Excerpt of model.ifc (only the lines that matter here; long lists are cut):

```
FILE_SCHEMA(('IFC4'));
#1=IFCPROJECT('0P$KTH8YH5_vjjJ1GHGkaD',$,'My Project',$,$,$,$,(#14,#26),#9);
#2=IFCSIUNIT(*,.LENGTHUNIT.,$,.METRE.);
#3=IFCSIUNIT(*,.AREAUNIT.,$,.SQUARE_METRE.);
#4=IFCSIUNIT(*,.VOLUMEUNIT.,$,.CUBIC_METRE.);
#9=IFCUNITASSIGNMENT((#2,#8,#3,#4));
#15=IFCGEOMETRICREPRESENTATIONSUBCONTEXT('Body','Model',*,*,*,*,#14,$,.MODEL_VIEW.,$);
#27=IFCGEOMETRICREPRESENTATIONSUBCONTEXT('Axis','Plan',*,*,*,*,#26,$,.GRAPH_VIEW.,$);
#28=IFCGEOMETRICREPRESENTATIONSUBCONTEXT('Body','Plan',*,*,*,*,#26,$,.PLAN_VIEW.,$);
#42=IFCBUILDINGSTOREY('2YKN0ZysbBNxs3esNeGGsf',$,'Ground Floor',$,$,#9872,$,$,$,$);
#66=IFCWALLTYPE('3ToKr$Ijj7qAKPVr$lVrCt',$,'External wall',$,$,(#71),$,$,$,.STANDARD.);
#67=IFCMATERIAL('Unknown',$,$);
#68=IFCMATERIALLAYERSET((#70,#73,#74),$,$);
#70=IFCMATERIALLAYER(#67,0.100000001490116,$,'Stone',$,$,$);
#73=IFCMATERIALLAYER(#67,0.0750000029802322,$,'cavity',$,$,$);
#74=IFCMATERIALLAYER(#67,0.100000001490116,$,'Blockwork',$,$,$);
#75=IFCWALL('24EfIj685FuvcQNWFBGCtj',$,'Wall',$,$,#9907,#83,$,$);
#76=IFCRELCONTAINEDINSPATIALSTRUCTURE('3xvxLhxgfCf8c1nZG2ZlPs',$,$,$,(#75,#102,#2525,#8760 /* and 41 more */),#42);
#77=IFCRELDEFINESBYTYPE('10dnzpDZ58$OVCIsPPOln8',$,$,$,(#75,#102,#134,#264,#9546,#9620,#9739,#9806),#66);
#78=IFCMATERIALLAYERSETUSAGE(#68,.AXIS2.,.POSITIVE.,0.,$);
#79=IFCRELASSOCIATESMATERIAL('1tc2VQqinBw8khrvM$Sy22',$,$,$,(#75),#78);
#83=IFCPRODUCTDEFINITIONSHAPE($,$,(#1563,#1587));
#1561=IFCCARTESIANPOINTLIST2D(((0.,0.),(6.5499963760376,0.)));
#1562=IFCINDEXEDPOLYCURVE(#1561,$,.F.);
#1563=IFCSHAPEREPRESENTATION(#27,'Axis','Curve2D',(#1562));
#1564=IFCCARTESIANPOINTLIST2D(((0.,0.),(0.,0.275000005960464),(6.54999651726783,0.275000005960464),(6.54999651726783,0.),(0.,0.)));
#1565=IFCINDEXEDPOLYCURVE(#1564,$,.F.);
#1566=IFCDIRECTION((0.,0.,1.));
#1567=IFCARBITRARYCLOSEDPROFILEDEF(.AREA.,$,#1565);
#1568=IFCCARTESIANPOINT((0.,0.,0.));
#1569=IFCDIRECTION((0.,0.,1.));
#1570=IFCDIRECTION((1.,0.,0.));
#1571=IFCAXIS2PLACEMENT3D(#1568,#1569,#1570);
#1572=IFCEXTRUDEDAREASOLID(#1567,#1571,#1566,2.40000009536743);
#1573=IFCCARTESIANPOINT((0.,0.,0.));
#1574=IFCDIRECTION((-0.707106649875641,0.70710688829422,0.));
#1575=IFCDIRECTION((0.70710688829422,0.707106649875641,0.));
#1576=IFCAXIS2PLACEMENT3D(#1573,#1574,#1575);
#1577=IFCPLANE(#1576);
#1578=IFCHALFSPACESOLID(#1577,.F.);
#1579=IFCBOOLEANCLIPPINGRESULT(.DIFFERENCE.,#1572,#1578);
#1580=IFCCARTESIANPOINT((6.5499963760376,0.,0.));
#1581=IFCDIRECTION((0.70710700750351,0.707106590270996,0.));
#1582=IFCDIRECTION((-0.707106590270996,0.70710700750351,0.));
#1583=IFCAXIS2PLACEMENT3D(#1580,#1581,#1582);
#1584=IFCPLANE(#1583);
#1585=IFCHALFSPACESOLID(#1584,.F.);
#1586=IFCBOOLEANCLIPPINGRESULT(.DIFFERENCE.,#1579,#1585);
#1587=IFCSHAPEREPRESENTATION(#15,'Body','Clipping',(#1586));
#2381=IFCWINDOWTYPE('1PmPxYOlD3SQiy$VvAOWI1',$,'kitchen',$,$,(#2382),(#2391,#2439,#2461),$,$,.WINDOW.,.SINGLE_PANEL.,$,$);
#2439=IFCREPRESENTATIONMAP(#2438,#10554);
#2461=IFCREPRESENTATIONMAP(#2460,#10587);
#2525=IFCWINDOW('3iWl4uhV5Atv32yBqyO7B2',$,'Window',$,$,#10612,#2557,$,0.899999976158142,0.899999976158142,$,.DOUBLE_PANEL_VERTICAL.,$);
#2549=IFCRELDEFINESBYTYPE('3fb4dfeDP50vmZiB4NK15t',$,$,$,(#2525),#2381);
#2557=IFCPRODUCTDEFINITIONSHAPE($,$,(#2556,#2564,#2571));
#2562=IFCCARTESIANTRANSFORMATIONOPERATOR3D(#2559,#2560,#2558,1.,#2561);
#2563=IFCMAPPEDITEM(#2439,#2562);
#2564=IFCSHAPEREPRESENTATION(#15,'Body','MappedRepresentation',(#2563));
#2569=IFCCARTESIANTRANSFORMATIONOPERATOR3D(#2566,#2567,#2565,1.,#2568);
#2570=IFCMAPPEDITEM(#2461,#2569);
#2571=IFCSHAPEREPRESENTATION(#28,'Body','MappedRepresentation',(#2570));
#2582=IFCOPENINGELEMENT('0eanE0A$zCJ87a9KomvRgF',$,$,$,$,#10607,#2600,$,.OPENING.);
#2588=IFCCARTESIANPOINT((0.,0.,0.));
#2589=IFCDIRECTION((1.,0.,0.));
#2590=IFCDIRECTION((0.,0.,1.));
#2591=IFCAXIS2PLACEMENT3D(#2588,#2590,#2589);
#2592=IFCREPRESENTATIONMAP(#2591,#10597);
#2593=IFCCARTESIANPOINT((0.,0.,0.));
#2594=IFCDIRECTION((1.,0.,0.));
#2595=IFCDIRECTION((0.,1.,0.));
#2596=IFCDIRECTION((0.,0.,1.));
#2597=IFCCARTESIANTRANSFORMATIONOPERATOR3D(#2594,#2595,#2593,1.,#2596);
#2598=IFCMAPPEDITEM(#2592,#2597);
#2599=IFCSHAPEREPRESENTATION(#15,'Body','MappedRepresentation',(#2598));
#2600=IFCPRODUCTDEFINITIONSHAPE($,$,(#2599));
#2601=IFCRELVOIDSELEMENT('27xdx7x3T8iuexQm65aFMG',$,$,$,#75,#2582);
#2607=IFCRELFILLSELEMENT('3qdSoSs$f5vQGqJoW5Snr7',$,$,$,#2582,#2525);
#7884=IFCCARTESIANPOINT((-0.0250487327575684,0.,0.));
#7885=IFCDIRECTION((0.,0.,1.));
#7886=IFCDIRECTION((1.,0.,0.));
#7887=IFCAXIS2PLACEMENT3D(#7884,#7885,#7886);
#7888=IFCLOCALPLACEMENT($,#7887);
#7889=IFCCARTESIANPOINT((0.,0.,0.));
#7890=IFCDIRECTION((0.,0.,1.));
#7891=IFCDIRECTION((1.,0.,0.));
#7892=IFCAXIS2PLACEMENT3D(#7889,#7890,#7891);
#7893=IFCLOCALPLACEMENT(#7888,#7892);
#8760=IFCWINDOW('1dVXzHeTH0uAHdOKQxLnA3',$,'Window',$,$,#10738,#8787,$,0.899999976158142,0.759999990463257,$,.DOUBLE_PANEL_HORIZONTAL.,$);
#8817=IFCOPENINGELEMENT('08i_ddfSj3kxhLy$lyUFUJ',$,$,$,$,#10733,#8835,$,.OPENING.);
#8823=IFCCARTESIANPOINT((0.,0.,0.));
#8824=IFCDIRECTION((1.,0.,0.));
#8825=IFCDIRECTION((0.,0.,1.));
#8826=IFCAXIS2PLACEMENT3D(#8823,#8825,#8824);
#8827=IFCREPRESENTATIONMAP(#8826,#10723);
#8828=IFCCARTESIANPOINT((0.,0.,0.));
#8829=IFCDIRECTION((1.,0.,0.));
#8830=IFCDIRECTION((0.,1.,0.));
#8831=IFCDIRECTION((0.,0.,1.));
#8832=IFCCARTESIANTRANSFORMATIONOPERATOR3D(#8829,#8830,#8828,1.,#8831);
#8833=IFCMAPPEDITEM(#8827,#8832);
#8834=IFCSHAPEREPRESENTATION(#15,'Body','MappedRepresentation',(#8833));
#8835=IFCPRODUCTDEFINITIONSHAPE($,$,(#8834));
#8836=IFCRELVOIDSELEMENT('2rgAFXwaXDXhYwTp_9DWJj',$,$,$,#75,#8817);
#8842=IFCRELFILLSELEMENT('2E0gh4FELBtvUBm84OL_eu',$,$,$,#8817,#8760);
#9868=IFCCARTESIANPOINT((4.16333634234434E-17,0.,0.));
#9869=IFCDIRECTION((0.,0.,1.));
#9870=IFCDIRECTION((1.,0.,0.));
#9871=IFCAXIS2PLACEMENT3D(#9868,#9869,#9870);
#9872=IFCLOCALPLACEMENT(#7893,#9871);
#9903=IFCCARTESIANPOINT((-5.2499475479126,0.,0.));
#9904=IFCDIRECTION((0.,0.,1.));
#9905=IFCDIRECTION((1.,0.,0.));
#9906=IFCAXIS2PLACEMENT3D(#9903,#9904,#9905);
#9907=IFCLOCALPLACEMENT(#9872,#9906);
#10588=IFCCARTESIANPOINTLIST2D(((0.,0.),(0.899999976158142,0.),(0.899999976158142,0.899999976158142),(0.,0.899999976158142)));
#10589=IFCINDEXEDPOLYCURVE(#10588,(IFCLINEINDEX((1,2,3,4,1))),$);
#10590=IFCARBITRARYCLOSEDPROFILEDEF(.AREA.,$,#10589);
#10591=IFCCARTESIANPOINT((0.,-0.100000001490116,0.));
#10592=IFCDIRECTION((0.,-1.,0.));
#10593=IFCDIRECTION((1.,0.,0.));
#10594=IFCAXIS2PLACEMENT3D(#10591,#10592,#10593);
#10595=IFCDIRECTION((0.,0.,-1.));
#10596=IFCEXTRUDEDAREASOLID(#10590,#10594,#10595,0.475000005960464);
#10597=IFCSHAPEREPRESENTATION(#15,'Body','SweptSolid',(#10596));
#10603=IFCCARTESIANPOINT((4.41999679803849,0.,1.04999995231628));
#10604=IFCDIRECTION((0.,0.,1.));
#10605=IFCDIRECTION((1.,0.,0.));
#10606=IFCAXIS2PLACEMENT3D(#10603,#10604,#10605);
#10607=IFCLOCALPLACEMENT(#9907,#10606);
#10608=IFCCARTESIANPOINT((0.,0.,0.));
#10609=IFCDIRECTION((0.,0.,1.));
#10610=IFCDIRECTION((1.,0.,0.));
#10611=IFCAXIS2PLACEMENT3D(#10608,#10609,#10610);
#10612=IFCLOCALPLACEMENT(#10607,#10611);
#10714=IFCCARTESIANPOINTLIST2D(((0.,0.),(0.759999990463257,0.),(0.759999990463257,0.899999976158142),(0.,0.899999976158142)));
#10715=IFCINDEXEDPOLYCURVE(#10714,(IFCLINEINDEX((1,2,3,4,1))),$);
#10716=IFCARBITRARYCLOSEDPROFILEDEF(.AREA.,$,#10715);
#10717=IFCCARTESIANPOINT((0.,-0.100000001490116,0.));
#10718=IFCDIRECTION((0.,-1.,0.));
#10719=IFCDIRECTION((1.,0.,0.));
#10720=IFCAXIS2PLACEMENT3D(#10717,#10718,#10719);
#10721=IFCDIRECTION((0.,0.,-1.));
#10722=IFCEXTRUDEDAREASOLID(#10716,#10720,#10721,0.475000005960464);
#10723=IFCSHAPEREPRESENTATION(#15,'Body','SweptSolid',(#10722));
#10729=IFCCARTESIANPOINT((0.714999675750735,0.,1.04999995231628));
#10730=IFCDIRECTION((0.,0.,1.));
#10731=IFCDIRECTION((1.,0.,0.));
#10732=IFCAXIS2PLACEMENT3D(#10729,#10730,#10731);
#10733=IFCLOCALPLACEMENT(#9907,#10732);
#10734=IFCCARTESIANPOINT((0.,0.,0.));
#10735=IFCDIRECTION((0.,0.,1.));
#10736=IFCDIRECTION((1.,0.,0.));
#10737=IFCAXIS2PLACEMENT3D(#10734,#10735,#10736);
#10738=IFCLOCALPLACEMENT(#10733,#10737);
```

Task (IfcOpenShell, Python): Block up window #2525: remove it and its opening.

```python
import ifcopenshell
import ifcopenshell.api.feature
import ifcopenshell.api.root
import ifcopenshell.geom
import ifcopenshell.util.shape

model = ifcopenshell.open("model.ifc")
settings = ifcopenshell.geom.settings()


def volume(element):
    """Net volume in cubic metres, openings subtracted."""
    shape = ifcopenshell.geom.create_shape(settings, element)
    return ifcopenshell.util.shape.get_volume(shape.geometry)


window = model.by_id(2525)
opening = window.FillsVoids[0].RelatingOpeningElement
wall = opening.VoidsElements[0].RelatingBuildingElement
before = volume(wall)

ifcopenshell.api.root.remove_product(model, product=window)
ifcopenshell.api.feature.remove_feature(model, feature=opening)

after = volume(wall)

print(f"wall volume {before:.3f} -> {after:.3f} m3")

model.write("model_v2.ifc")
```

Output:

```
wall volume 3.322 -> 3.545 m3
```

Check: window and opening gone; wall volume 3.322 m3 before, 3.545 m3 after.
